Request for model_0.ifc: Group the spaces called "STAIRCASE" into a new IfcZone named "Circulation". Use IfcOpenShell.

First a look at what the model holds.

```python
import ifcopenshell

model = ifcopenshell.open("model_0.ifc")
print(model.schema)
seen = {}
for space in model.by_type("IfcSpace"):
    seen[space.LongName] = seen.get(space.LongName, 0) + 1
for name, count in sorted(seen.items(), key=str):
    print(count, "x", name)
print("zones:", [z.Name for z in model.by_type("IfcZone")][:20])
```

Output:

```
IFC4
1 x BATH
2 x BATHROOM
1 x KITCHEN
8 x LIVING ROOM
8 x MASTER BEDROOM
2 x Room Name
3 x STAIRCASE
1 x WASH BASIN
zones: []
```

```python
import ifcopenshell
import ifcopenshell.api.group
import ifcopenshell.api.root

model = ifcopenshell.open("model_0.ifc")

names = {"STAIRCASE"}
spaces = [s for s in model.by_type("IfcSpace") if s.LongName in names]

zone = ifcopenshell.api.root.create_entity(model, ifc_class="IfcZone", name="Circulation")
ifcopenshell.api.group.assign_group(model, products=spaces, group=zone)
print(len(spaces), "spaces in", zone.Name)

model.write("model_0-out.ifc")
```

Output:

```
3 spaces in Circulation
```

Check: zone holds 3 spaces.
